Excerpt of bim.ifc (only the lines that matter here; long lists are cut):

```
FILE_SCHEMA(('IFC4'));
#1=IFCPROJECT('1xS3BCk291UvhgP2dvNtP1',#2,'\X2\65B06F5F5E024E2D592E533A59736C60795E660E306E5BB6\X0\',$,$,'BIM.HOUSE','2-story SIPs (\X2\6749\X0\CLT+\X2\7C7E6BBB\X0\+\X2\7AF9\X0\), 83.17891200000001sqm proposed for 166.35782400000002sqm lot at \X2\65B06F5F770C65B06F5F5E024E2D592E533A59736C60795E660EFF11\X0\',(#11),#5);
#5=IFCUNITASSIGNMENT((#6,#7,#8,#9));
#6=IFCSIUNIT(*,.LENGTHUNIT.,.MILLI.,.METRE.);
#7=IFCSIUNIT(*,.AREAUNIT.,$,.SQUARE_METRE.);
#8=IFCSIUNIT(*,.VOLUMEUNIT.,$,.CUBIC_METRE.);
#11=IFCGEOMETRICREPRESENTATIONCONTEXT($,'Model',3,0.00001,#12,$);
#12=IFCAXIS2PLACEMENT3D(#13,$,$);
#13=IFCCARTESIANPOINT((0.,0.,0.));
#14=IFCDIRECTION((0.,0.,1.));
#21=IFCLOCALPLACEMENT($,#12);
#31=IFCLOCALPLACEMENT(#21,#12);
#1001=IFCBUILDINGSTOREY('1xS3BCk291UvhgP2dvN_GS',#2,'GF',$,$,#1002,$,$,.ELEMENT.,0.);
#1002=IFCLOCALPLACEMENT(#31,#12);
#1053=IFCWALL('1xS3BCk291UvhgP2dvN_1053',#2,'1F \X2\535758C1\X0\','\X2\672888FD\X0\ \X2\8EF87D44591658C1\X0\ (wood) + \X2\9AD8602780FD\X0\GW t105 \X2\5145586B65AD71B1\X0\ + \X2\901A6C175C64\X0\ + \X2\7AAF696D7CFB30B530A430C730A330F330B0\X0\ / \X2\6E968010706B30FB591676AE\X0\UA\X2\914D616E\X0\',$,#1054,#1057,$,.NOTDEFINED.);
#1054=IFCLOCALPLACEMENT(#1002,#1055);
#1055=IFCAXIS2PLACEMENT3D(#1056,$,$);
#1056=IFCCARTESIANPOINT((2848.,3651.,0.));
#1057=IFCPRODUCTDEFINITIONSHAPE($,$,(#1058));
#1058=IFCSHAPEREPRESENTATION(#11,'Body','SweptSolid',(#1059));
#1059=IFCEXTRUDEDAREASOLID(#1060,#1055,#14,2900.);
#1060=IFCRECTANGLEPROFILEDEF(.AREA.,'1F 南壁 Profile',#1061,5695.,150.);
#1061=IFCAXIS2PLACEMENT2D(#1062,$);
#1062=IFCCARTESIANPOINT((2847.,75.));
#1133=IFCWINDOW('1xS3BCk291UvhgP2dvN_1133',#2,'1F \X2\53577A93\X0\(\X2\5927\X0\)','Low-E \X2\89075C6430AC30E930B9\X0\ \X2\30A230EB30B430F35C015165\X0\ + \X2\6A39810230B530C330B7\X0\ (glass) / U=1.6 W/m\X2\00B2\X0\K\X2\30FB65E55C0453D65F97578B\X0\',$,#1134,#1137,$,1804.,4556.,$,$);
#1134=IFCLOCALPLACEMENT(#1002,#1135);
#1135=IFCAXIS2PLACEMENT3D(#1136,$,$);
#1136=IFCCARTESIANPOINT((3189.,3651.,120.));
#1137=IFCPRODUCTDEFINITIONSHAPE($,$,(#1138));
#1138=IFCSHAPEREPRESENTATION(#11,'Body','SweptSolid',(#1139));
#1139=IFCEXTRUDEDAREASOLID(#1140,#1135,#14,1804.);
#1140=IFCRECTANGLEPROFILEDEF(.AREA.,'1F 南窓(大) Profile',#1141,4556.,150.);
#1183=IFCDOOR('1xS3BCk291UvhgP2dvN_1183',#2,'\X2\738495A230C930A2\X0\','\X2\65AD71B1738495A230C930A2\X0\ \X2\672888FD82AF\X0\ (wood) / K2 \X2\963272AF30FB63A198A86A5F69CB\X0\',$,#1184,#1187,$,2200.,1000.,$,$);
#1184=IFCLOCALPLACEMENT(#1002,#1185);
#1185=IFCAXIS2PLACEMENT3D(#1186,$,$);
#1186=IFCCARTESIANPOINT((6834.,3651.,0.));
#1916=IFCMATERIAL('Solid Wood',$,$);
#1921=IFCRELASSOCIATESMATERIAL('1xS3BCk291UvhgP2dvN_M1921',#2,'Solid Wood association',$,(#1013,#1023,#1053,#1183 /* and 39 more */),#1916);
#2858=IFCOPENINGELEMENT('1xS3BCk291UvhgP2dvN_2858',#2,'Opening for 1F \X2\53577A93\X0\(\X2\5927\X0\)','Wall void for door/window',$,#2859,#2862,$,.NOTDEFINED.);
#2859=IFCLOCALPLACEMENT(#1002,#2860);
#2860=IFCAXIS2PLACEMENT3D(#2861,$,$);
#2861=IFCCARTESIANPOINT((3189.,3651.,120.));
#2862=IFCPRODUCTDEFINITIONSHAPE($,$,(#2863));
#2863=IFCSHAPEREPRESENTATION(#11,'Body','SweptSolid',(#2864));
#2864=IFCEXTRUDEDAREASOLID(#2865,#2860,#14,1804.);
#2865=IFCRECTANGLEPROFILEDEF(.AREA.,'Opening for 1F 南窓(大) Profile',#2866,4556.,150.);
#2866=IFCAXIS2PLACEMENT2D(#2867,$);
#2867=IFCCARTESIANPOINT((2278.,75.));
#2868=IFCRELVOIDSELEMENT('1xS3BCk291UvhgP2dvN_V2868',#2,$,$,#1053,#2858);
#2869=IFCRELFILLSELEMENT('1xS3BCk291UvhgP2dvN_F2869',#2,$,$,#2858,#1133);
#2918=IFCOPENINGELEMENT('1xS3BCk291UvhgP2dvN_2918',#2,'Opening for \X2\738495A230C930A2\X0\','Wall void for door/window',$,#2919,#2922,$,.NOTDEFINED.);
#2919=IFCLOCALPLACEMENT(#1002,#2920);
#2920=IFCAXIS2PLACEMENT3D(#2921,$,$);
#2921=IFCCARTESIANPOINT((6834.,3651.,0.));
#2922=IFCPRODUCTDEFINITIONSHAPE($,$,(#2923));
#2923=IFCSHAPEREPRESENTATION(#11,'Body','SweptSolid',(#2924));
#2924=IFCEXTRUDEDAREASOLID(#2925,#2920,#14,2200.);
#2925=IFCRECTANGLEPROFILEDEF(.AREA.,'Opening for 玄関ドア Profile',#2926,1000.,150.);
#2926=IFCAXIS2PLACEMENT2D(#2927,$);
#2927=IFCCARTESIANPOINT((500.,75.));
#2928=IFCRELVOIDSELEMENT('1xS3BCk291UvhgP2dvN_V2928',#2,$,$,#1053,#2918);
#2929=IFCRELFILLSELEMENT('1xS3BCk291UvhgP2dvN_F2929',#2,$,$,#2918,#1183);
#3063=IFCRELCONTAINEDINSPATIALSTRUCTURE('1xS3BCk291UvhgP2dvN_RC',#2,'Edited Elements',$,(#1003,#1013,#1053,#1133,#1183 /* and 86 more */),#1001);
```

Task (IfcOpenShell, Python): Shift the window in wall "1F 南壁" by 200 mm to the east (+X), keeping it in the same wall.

```python
import ifcopenshell
import ifcopenshell.api.geometry
import ifcopenshell.util.placement
import ifcopenshell.util.unit

model = ifcopenshell.open("bim.ifc")
unit_scale = ifcopenshell.util.unit.calculate_unit_scale(model)

window = model.by_guid("1xS3BCk291UvhgP2dvN_1133")
opening = window.FillsVoids[0].RelatingOpeningElement
wall = opening.VoidsElements[0].RelatingBuildingElement

wall_matrix = ifcopenshell.util.placement.get_local_placement(wall.ObjectPlacement)
shift = wall_matrix[:3, 0] * 0.2 / unit_scale
before = ifcopenshell.util.placement.get_local_placement(window.ObjectPlacement)[:3, 3].copy()

# The window is not placed relative to its opening, so move both.
for product in (opening, window):
    matrix = ifcopenshell.util.placement.get_local_placement(product.ObjectPlacement)
    matrix[:3, 3] += shift
    ifcopenshell.api.geometry.edit_object_placement(model, product=product, matrix=matrix, is_si=False)

after = ifcopenshell.util.placement.get_local_placement(window.ObjectPlacement)[:3, 3]
print("window moved by", (after - before).round(3) + 0.0)

model.write("bim_updated.ifc")
```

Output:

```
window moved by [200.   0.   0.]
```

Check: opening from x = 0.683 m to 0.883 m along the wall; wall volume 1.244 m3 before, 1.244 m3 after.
